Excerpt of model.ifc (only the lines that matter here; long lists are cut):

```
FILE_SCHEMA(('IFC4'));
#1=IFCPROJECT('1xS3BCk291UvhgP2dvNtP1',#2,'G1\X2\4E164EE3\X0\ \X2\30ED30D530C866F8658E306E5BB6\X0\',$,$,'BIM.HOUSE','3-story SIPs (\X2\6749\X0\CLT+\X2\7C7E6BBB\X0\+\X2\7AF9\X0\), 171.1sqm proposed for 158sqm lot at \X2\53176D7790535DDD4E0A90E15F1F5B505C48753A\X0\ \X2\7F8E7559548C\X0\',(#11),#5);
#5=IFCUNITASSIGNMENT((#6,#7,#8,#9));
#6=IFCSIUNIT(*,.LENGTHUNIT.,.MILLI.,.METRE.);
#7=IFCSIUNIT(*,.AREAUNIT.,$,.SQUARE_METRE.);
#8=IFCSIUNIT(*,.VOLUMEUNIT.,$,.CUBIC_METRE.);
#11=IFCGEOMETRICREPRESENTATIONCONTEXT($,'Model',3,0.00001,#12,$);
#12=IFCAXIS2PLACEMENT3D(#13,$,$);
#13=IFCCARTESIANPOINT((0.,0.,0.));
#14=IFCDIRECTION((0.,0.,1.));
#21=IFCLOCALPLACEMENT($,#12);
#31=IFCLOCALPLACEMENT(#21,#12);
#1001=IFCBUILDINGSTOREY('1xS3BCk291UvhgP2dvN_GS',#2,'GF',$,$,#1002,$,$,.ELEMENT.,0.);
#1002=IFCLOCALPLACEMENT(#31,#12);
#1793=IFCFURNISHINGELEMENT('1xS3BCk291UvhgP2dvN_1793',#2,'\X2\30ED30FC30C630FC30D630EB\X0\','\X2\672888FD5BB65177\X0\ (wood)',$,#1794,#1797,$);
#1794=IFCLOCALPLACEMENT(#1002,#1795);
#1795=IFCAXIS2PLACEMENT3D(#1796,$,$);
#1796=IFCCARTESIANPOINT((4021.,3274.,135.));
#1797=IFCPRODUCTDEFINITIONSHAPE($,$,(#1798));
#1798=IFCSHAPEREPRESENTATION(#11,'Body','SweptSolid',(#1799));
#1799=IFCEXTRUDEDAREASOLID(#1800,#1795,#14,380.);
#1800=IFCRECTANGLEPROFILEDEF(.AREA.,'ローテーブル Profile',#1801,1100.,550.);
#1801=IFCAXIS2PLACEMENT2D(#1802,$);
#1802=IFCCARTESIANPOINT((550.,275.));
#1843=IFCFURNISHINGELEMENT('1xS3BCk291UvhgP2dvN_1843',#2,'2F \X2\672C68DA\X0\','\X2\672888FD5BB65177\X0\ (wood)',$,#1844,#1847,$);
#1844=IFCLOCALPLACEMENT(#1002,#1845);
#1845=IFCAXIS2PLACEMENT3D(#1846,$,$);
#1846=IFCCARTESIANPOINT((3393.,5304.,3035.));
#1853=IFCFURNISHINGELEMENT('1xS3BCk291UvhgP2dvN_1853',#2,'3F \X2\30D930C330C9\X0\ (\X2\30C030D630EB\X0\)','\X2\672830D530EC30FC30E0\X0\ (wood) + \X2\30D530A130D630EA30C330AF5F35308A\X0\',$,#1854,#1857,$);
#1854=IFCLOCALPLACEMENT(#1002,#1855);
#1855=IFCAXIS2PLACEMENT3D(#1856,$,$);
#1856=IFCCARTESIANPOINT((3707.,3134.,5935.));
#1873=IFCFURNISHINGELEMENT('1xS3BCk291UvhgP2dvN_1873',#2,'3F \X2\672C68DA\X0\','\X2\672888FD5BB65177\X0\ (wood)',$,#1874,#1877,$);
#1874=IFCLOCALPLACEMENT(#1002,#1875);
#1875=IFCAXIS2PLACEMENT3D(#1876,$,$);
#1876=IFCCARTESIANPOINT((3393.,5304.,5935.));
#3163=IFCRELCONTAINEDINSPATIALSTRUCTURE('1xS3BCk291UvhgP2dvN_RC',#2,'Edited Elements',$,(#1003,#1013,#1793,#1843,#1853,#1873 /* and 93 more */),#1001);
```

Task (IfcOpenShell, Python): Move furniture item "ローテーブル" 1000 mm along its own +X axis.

```python
import ifcopenshell
import ifcopenshell.api.geometry
import ifcopenshell.util.placement

model = ifcopenshell.open("model.ifc")

item = model.by_id(1793)
matrix = ifcopenshell.util.placement.get_local_placement(item.ObjectPlacement)
matrix[:3, 3] += matrix[:3, 0] * 1000.0
ifcopenshell.api.geometry.edit_object_placement(model, product=item, matrix=matrix, is_si=False)

print(ifcopenshell.util.placement.get_local_placement(item.ObjectPlacement).round(3) + 0.0)

model.write("model_v2.ifc")
```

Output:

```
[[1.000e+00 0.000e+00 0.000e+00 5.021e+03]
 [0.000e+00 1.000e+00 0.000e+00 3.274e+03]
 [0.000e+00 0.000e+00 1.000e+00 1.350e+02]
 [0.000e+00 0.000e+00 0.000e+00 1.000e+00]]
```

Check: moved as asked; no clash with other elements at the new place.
